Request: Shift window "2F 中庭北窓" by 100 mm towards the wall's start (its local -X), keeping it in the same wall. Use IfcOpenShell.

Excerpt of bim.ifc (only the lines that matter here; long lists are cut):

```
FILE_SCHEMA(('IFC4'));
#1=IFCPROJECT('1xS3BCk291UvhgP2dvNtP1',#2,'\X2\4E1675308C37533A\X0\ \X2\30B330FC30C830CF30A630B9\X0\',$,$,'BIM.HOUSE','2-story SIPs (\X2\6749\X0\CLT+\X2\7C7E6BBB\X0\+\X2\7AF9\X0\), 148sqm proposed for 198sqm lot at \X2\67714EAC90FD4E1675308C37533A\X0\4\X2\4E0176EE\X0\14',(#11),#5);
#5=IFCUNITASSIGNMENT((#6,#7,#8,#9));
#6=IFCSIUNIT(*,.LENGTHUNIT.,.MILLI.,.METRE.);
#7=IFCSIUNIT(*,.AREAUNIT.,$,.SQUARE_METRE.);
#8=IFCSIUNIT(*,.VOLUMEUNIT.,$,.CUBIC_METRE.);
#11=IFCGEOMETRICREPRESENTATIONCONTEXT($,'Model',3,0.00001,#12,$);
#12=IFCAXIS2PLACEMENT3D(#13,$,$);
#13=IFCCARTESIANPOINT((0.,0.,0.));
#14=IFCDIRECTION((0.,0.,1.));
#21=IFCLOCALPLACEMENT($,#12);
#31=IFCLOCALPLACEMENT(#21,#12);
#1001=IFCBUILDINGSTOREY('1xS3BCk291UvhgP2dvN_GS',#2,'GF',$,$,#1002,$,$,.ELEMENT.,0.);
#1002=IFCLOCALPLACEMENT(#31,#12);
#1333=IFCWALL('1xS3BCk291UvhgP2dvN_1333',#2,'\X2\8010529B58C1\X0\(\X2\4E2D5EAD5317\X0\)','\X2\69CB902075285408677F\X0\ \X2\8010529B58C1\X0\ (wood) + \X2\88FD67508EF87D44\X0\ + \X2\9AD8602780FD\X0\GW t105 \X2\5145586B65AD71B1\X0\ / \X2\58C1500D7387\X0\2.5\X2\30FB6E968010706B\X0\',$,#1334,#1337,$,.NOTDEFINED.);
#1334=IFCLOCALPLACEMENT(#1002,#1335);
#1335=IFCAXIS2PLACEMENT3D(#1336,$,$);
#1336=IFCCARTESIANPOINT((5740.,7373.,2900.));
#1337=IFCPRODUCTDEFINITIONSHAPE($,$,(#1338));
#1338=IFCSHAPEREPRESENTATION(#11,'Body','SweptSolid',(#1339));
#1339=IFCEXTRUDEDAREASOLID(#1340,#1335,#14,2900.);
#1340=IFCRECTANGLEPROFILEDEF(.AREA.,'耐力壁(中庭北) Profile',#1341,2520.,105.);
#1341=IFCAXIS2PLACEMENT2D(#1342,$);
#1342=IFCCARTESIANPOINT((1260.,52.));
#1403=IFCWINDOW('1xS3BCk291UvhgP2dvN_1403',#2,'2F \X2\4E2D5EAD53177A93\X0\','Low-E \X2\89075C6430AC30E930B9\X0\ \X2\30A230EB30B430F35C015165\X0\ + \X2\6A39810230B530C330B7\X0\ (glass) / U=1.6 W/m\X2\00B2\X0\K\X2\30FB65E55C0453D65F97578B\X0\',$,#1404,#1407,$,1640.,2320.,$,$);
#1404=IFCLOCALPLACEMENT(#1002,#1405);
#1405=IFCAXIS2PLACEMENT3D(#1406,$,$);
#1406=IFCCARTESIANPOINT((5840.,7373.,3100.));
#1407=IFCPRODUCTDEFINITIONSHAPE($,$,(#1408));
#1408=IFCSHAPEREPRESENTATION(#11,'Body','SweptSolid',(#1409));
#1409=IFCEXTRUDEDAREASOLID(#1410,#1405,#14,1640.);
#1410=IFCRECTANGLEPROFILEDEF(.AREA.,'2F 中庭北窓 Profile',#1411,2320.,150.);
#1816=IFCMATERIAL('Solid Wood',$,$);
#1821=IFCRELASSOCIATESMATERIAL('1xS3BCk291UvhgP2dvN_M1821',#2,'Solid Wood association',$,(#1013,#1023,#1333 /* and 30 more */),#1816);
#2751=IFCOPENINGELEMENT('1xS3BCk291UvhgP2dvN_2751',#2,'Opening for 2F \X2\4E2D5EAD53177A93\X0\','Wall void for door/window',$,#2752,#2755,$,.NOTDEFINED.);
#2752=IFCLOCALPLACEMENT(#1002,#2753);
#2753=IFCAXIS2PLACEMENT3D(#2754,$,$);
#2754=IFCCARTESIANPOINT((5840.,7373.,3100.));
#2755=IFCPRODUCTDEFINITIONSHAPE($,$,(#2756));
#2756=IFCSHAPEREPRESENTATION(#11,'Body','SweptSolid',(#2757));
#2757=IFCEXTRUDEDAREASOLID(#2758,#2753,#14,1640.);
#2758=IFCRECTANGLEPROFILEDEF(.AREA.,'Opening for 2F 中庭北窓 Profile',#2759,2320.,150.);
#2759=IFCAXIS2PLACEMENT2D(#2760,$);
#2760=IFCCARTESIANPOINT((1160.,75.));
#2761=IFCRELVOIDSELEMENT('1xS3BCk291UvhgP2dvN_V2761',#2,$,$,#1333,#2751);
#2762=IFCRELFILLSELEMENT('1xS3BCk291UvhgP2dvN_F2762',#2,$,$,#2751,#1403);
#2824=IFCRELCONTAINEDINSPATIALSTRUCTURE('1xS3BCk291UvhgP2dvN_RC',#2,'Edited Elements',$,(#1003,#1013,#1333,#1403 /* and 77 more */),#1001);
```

```python
import ifcopenshell
import ifcopenshell.api.geometry
import ifcopenshell.util.placement

model = ifcopenshell.open("bim.ifc")

window = model.by_id(1403)
opening = window.FillsVoids[0].RelatingOpeningElement
wall = opening.VoidsElements[0].RelatingBuildingElement

wall_matrix = ifcopenshell.util.placement.get_local_placement(wall.ObjectPlacement)
shift = wall_matrix[:3, 0] * -100.0
before = ifcopenshell.util.placement.get_local_placement(window.ObjectPlacement)[:3, 3].copy()

# The window is not placed relative to its opening, so move both.
for product in (opening, window):
    matrix = ifcopenshell.util.placement.get_local_placement(product.ObjectPlacement)
    matrix[:3, 3] += shift
    ifcopenshell.api.geometry.edit_object_placement(model, product=product, matrix=matrix, is_si=False)

after = ifcopenshell.util.placement.get_local_placement(window.ObjectPlacement)[:3, 3]
print("window moved by", (after - before).round(3) + 0.0)

model.write("bim_edited.ifc")
```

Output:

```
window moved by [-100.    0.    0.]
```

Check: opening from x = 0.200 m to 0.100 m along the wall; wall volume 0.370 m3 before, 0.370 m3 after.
